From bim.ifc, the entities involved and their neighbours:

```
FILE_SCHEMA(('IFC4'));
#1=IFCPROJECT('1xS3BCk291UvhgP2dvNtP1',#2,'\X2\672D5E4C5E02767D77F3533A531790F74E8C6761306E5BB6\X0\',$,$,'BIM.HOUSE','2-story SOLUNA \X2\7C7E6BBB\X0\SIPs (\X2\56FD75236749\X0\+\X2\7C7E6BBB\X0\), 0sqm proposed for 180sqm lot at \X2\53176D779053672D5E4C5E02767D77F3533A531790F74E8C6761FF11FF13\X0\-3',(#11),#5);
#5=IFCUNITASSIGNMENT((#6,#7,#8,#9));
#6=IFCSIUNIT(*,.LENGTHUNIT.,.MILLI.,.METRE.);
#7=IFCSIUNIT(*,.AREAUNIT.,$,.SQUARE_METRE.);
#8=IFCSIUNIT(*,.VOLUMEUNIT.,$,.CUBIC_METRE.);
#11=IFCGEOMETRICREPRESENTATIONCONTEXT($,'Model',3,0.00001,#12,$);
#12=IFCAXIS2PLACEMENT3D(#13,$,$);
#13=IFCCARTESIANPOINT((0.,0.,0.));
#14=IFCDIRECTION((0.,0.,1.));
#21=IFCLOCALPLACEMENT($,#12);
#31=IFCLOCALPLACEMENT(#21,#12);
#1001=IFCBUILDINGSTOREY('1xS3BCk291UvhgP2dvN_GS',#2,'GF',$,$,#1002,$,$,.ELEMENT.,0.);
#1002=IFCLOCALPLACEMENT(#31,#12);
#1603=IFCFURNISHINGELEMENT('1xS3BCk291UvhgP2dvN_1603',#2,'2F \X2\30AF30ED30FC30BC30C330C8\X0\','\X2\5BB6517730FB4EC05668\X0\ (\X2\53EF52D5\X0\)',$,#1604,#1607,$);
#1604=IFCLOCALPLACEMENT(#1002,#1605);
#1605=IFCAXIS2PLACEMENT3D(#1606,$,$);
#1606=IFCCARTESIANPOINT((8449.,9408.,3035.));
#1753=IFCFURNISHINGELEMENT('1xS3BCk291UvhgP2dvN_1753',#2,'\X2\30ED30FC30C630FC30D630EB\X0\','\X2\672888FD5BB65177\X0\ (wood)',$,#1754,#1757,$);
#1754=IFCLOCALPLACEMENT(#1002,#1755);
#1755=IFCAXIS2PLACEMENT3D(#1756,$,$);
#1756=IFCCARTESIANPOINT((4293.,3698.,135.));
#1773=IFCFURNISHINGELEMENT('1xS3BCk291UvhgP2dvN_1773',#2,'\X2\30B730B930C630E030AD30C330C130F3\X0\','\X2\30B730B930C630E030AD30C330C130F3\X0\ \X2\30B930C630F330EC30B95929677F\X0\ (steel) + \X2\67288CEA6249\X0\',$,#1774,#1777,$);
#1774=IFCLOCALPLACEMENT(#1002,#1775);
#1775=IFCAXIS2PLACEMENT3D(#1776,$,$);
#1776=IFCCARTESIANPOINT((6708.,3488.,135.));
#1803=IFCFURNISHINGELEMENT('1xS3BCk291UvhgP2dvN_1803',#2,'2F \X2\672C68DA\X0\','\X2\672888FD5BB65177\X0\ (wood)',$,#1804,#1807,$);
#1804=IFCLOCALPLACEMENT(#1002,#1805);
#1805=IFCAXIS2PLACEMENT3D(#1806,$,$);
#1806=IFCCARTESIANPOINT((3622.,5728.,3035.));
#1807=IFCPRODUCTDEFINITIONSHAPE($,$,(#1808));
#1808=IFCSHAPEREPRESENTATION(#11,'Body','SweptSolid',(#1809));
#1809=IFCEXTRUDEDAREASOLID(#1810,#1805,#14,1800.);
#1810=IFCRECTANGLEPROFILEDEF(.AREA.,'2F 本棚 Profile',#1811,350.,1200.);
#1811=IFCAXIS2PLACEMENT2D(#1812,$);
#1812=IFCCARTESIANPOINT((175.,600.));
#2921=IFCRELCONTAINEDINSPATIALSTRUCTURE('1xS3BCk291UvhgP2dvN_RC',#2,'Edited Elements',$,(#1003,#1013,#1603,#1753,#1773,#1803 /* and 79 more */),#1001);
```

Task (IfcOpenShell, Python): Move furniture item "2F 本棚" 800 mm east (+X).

```python
import ifcopenshell
import ifcopenshell.api.geometry
import ifcopenshell.util.placement
import ifcopenshell.util.unit

model = ifcopenshell.open("bim.ifc")
unit_scale = ifcopenshell.util.unit.calculate_unit_scale(model)

item = model.by_guid("1xS3BCk291UvhgP2dvN_1803")
matrix = ifcopenshell.util.placement.get_local_placement(item.ObjectPlacement)
matrix[0, 3] += 0.8 / unit_scale
ifcopenshell.api.geometry.edit_object_placement(model, product=item, matrix=matrix, is_si=False)

print(ifcopenshell.util.placement.get_local_placement(item.ObjectPlacement).round(3) + 0.0)

model.write("bim_edited.ifc")
```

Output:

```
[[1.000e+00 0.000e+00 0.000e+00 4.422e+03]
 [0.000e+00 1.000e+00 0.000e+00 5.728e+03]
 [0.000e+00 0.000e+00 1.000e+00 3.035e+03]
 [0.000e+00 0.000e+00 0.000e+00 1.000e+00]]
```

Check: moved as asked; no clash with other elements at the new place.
